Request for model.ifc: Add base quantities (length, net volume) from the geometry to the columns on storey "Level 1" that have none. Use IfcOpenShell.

First a look at what the model holds.

```python
import ifcopenshell
import ifcopenshell.util.element
import ifcopenshell.util.unit

model = ifcopenshell.open("model.ifc")
print(model.schema)
for unit_type in ("LENGTHUNIT", "AREAUNIT", "VOLUMEUNIT"):
    print(unit_type, ifcopenshell.util.unit.calculate_unit_scale(model, unit_type))
storey = next(s for s in model.by_type("IfcBuildingStorey") if s.Name == "Level 1")
columns = [e for e in ifcopenshell.util.element.get_decomposition(storey) if e.is_a("IfcColumn")]
for e in sorted(columns, key=lambda e: e.id()):
    print(e.id(), e.is_a(), e.Name, list(ifcopenshell.util.element.get_psets(e, qtos_only=True)), sep=" | ")
```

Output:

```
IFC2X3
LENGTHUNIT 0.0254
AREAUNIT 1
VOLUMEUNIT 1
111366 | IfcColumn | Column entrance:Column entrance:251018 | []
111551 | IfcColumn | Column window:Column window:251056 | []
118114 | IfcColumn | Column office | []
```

```python
import ifcopenshell
import ifcopenshell.api.pset
import ifcopenshell.geom
import ifcopenshell.util.element
import ifcopenshell.util.shape
import ifcopenshell.util.unit

model = ifcopenshell.open("model.ifc")
unit_scale = ifcopenshell.util.unit.calculate_unit_scale(model)
volume_scale = ifcopenshell.util.unit.calculate_unit_scale(model, "VOLUMEUNIT")
settings = ifcopenshell.geom.settings()

storey = next(s for s in model.by_type("IfcBuildingStorey") if s.Name == "Level 1")
columns = [e for e in ifcopenshell.util.element.get_decomposition(storey) if e.is_a("IfcColumn")]

for e in sorted(columns, key=lambda e: e.id()):
    if ifcopenshell.util.element.get_psets(e, qtos_only=True, should_inherit=False):
        continue
    # Geometry comes back in metres, in the element's own axes.
    shape = ifcopenshell.geom.create_shape(settings, e)
    values = {
        "Length": ifcopenshell.util.shape.get_z(shape.geometry) / unit_scale,
        "NetVolume": ifcopenshell.util.shape.get_volume(shape.geometry) / volume_scale,
    }
    qto = ifcopenshell.api.pset.add_qto(model, product=e, name="BaseQuantities")
    ifcopenshell.api.pset.edit_qto(model, qto=qto, properties=values)
    print(e.id(), {k: round(v, 3) for k, v in values.items()})

model.write("model_edited.ifc")
```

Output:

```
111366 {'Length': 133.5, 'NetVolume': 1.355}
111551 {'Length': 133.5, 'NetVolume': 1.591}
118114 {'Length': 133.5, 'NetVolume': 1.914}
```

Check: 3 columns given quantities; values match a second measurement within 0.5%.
